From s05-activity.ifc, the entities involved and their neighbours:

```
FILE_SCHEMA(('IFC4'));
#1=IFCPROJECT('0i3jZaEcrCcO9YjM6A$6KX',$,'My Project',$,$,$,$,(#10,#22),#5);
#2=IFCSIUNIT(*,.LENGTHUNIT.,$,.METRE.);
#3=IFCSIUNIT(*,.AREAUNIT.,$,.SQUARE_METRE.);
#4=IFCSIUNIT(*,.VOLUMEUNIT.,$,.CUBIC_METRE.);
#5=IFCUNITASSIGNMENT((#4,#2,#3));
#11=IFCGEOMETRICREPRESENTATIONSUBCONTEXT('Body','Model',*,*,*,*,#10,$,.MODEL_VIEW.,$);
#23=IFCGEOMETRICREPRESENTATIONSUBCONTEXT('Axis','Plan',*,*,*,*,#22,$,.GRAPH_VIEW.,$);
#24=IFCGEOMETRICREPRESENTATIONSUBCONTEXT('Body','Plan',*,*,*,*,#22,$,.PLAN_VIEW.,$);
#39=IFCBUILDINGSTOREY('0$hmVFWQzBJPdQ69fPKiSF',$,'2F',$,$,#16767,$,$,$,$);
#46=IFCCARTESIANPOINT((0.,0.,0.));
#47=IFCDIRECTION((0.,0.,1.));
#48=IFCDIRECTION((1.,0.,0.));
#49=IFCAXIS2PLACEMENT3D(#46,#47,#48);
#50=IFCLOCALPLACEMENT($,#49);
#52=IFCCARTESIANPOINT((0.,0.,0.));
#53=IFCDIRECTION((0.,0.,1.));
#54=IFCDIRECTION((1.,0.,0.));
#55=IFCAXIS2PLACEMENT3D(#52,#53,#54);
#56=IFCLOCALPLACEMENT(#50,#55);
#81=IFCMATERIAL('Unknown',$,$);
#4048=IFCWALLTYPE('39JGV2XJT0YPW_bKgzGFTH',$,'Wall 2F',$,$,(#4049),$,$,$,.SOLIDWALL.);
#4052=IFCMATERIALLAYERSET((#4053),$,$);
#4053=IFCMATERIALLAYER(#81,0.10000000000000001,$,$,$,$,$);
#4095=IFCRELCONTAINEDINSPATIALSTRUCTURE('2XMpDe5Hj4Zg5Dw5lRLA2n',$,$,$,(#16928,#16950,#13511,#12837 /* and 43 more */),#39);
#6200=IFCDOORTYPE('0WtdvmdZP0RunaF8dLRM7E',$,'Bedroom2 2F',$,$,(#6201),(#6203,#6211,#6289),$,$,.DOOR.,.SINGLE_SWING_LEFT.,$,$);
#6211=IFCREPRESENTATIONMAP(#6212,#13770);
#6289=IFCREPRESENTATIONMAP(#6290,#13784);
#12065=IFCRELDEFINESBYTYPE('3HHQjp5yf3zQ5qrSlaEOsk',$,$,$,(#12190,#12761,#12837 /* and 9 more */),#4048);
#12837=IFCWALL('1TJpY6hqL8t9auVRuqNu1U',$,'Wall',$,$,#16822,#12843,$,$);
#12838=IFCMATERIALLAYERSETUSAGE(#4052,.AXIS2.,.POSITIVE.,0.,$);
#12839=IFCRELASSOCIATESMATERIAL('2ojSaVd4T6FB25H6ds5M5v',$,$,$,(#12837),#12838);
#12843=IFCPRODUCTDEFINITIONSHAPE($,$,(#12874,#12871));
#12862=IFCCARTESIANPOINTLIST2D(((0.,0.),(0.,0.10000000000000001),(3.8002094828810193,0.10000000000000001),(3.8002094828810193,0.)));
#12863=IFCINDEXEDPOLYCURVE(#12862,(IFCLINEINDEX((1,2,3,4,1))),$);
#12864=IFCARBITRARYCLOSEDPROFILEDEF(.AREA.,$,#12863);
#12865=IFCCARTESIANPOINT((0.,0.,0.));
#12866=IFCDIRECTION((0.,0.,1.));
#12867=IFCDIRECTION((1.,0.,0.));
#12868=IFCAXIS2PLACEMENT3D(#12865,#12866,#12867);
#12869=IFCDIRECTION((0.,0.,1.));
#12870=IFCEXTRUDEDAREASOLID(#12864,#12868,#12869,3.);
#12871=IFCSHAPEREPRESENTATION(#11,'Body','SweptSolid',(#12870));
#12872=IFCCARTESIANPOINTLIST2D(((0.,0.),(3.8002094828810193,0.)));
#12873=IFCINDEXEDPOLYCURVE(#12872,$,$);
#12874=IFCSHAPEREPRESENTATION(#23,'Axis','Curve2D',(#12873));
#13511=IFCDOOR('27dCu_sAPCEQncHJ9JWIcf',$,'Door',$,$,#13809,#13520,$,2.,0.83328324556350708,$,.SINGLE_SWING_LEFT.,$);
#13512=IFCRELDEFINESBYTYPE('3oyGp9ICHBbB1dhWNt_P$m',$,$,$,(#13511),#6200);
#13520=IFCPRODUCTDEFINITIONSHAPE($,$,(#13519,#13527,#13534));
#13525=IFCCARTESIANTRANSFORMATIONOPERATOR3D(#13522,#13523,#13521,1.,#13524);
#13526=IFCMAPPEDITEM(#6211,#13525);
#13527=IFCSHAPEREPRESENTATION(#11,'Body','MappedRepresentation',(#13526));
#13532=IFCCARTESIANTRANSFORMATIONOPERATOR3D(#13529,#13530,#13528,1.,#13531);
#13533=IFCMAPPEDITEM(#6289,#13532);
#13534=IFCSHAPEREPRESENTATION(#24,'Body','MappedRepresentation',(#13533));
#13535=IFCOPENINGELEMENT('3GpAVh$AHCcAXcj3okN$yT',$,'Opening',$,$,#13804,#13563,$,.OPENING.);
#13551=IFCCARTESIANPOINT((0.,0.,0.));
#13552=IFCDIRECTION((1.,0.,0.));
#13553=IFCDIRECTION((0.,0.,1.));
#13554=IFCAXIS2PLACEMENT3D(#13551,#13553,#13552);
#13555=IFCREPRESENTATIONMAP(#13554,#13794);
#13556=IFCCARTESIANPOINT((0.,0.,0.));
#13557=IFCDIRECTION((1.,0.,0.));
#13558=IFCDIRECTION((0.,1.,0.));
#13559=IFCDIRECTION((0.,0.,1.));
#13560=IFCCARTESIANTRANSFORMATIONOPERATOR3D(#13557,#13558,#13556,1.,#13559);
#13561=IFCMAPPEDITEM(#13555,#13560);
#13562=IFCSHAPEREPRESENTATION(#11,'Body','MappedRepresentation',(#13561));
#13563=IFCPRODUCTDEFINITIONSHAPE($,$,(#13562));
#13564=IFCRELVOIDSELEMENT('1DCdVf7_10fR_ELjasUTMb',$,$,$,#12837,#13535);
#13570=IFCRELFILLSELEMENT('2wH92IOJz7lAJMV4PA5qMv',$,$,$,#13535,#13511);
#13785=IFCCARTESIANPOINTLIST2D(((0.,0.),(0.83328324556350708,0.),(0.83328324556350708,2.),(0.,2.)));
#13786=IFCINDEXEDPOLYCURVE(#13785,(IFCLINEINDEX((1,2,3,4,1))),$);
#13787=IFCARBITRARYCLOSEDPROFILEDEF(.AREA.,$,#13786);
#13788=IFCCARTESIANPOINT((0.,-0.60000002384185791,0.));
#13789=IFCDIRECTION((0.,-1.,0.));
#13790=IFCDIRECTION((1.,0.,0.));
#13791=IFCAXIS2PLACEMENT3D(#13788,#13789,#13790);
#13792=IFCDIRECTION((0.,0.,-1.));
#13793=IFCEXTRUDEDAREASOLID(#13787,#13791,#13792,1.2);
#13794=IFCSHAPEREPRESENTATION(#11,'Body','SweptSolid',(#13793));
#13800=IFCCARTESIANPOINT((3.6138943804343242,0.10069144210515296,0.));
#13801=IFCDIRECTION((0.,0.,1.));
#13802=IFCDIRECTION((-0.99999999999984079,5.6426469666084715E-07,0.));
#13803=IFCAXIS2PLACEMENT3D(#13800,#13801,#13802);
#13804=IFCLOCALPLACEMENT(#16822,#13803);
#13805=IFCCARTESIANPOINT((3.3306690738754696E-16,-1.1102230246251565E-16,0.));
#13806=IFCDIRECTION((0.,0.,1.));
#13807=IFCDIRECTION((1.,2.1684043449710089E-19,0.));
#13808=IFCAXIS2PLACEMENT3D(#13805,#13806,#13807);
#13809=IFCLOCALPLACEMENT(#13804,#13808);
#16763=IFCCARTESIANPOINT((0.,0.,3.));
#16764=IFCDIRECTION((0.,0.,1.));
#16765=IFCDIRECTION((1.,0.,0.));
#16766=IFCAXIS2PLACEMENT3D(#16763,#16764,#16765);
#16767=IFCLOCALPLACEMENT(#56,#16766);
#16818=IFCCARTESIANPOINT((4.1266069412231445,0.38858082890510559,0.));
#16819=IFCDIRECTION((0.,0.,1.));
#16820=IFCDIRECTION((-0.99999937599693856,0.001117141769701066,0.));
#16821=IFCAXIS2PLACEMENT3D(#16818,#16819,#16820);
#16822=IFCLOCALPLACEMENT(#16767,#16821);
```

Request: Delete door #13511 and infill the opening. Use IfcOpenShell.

```python
import ifcopenshell
import ifcopenshell.api.feature
import ifcopenshell.api.root
import ifcopenshell.geom
import ifcopenshell.util.shape

model = ifcopenshell.open("s05-activity.ifc")
settings = ifcopenshell.geom.settings()


def volume(element):
    """Net volume in cubic metres, openings subtracted."""
    shape = ifcopenshell.geom.create_shape(settings, element)
    return ifcopenshell.util.shape.get_volume(shape.geometry)


door = model.by_id(13511)
opening = door.FillsVoids[0].RelatingOpeningElement
wall = opening.VoidsElements[0].RelatingBuildingElement
before = volume(wall)

ifcopenshell.api.root.remove_product(model, product=door)
ifcopenshell.api.feature.remove_feature(model, feature=opening)

after = volume(wall)

print(f"wall volume {before:.3f} -> {after:.3f} m3")

model.write("s05-activity_rev.ifc")
```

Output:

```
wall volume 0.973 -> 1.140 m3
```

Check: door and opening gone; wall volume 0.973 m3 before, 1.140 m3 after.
